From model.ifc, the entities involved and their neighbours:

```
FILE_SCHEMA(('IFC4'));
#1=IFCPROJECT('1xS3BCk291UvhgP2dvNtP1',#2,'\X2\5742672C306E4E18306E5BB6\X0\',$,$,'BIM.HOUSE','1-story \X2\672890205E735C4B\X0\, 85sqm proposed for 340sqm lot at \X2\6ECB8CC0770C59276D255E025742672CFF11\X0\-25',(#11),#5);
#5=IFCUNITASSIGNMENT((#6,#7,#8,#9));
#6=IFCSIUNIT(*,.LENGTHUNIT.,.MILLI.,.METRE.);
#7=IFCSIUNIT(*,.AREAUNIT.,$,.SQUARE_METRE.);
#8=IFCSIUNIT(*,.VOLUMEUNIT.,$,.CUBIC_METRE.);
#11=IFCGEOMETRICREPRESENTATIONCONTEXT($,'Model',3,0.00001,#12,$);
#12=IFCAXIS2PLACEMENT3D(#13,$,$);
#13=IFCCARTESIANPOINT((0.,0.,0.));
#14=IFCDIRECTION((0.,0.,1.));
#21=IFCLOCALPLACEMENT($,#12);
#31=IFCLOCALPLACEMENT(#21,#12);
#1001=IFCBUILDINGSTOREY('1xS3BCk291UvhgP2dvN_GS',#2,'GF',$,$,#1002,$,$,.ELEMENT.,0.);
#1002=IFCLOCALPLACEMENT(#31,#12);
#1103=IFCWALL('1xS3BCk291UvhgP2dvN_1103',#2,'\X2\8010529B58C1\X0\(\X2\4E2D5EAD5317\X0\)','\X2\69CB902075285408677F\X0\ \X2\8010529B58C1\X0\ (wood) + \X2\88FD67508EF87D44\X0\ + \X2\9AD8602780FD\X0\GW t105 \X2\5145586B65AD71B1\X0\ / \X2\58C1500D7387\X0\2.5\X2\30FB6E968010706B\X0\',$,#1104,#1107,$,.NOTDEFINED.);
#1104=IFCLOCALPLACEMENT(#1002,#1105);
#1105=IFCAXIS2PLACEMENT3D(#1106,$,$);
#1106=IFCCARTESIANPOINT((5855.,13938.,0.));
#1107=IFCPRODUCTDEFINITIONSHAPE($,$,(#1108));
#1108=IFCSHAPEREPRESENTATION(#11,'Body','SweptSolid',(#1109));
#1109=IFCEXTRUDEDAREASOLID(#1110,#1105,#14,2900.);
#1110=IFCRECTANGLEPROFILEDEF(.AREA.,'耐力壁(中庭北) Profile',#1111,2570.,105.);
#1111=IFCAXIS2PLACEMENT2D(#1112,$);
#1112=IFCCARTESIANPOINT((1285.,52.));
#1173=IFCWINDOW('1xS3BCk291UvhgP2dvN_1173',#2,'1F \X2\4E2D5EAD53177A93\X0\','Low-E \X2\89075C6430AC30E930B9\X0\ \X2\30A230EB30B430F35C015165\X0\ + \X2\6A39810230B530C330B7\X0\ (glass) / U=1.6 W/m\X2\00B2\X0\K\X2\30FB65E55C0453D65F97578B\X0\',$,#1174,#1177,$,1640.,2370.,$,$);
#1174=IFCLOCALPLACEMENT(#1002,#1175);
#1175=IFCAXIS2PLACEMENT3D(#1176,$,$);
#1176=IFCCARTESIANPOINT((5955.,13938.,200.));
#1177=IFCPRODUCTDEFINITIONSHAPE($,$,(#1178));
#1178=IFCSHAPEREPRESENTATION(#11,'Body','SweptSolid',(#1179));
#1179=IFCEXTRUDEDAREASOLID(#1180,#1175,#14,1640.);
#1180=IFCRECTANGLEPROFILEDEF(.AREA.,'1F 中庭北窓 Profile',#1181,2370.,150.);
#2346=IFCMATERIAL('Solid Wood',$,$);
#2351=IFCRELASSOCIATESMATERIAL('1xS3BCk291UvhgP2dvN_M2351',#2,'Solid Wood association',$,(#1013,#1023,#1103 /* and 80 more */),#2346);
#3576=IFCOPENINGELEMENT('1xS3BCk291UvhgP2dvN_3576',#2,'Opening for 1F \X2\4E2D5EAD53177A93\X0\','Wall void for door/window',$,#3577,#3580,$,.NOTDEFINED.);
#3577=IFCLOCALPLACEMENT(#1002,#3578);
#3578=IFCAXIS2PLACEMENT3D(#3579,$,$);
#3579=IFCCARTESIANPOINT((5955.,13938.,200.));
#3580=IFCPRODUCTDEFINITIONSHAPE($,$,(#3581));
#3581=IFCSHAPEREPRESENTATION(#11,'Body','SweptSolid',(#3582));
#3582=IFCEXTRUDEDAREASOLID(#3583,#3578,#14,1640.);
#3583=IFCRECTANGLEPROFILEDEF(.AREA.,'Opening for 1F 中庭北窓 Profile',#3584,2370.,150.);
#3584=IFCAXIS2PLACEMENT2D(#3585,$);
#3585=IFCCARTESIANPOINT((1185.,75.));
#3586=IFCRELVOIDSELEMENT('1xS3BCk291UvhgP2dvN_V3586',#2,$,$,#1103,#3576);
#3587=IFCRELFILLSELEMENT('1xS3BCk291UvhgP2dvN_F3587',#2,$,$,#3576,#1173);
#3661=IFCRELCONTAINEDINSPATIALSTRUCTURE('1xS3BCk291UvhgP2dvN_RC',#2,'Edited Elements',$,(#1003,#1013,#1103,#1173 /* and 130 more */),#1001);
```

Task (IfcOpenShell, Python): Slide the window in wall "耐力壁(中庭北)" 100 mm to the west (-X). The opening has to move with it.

```python
import ifcopenshell
import ifcopenshell.api.geometry
import ifcopenshell.util.placement

model = ifcopenshell.open("model.ifc")

window = model.by_guid("1xS3BCk291UvhgP2dvN_1173")
opening = window.FillsVoids[0].RelatingOpeningElement
wall = opening.VoidsElements[0].RelatingBuildingElement

wall_matrix = ifcopenshell.util.placement.get_local_placement(wall.ObjectPlacement)
shift = wall_matrix[:3, 0] * -100.0
before = ifcopenshell.util.placement.get_local_placement(window.ObjectPlacement)[:3, 3].copy()

# The window is not placed relative to its opening, so move both.
for product in (opening, window):
    matrix = ifcopenshell.util.placement.get_local_placement(product.ObjectPlacement)
    matrix[:3, 3] += shift
    ifcopenshell.api.geometry.edit_object_placement(model, product=product, matrix=matrix, is_si=False)

after = ifcopenshell.util.placement.get_local_placement(window.ObjectPlacement)[:3, 3]
print("window moved by", (after - before).round(3) + 0.0)

model.write("model-out.ifc")
```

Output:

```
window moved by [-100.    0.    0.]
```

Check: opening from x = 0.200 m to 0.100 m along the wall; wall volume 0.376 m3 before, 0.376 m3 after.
